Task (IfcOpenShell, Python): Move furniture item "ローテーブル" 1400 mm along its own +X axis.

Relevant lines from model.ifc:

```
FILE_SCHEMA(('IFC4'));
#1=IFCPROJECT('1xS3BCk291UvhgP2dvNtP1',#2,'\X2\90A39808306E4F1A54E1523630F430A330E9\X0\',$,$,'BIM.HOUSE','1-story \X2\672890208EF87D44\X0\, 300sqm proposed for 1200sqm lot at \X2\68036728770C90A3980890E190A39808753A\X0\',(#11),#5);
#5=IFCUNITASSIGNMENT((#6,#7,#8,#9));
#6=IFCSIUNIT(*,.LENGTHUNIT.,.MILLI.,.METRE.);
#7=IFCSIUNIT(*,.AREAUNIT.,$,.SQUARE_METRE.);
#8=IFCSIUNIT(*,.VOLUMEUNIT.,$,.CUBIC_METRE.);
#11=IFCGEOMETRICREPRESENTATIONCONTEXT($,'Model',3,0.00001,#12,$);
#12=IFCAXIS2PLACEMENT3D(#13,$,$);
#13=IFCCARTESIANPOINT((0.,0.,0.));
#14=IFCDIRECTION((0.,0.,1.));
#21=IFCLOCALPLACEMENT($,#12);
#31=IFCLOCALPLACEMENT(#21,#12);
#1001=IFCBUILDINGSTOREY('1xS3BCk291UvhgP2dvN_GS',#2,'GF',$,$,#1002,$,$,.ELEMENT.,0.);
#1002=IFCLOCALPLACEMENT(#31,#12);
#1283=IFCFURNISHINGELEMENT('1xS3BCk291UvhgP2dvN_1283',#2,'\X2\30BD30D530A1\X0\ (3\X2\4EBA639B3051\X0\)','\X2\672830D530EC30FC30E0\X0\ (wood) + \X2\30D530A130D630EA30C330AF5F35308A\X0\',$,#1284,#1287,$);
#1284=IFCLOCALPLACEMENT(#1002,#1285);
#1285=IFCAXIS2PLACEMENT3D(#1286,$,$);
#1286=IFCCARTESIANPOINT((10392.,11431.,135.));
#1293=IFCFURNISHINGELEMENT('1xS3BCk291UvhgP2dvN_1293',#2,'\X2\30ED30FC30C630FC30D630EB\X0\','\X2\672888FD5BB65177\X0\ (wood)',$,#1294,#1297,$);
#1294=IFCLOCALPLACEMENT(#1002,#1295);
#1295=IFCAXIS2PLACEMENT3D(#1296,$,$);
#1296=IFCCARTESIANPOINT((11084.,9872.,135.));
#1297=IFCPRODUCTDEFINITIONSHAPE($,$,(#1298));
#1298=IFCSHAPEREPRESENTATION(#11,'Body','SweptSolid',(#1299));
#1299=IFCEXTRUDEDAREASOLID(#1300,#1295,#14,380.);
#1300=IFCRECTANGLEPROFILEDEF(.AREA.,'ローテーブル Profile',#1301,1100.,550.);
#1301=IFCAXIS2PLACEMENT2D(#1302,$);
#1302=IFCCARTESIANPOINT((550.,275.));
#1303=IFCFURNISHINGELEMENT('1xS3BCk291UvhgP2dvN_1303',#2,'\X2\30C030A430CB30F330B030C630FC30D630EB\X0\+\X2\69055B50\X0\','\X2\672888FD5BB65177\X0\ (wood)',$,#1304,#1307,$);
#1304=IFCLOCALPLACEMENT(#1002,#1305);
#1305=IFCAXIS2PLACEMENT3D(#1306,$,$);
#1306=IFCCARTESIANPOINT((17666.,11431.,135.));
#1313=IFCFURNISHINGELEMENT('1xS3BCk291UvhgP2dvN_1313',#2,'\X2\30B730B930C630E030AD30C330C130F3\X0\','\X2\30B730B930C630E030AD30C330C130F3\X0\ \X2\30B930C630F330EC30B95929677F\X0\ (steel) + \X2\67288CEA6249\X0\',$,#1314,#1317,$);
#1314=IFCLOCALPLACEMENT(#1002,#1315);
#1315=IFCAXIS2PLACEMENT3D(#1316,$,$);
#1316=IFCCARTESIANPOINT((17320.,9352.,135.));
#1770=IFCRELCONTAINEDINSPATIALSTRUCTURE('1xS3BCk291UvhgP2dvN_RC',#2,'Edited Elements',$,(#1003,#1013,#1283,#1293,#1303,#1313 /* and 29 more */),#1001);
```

```python
import ifcopenshell
import ifcopenshell.api.geometry
import ifcopenshell.util.placement

model = ifcopenshell.open("model.ifc")

item = model.by_id(1293)
matrix = ifcopenshell.util.placement.get_local_placement(item.ObjectPlacement)
matrix[:3, 3] += matrix[:3, 0] * 1400.0
ifcopenshell.api.geometry.edit_object_placement(model, product=item, matrix=matrix, is_si=False)

print(ifcopenshell.util.placement.get_local_placement(item.ObjectPlacement).round(3) + 0.0)

model.write("model_rev.ifc")
```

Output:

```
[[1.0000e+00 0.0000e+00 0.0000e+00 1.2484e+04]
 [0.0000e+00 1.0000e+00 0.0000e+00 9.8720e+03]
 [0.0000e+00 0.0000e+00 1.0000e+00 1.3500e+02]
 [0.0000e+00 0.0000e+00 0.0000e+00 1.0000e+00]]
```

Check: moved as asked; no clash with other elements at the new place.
